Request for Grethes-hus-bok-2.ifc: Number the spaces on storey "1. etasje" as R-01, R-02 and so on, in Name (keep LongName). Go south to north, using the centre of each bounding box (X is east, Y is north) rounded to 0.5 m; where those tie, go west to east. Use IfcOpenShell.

First a look at what the model holds.

```python
import ifcopenshell
import ifcopenshell.util.element
import ifcopenshell.util.placement

model = ifcopenshell.open("Grethes-hus-bok-2.ifc")
print(model.schema)
storey = next(s for s in model.by_type("IfcBuildingStorey") if s.Name == "1. etasje")
spaces = [e for e in ifcopenshell.util.element.get_decomposition(storey) if e.is_a("IfcSpace")]
for e in sorted(spaces, key=lambda e: e.id()):
    origin = ifcopenshell.util.placement.get_local_placement(e.ObjectPlacement)[:3, 3]
    print(e.id(), e.Name, e.LongName, origin.round(2) + 0.0, sep=" | ")
```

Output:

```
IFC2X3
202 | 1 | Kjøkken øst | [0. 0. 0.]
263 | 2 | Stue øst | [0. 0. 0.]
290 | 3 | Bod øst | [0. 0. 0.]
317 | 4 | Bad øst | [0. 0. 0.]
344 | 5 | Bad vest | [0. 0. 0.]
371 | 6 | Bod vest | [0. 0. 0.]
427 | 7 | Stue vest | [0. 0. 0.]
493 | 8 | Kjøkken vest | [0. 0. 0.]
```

```python
import ifcopenshell
import ifcopenshell.geom
import ifcopenshell.util.element
import ifcopenshell.util.shape

model = ifcopenshell.open("Grethes-hus-bok-2.ifc")
settings = ifcopenshell.geom.settings()
settings.set("use-world-coords", True)


def centre(element):
    shape = ifcopenshell.geom.create_shape(settings, element)
    return ifcopenshell.util.shape.get_bbox_centroid(shape.geometry)


storey = next(s for s in model.by_type("IfcBuildingStorey") if s.Name == "1. etasje")
spaces = [e for e in ifcopenshell.util.element.get_decomposition(storey) if e.is_a("IfcSpace")]

# Insertion points can sit at a corner or the storey origin, so sort by the geometry (in metres).
centres = {e: centre(e) for e in spaces}
spaces.sort(key=lambda e: (round(centres[e][1] / 0.5), centres[e][0]))

for i, e in enumerate(spaces, start=1):
    number = f"R-{i:02d}"
    e.Name = number
    print(e.id(), number)

model.write("Grethes-hus-bok-2_rev.ifc")
```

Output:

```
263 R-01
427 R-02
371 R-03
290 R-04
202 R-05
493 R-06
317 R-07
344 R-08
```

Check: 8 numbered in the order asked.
